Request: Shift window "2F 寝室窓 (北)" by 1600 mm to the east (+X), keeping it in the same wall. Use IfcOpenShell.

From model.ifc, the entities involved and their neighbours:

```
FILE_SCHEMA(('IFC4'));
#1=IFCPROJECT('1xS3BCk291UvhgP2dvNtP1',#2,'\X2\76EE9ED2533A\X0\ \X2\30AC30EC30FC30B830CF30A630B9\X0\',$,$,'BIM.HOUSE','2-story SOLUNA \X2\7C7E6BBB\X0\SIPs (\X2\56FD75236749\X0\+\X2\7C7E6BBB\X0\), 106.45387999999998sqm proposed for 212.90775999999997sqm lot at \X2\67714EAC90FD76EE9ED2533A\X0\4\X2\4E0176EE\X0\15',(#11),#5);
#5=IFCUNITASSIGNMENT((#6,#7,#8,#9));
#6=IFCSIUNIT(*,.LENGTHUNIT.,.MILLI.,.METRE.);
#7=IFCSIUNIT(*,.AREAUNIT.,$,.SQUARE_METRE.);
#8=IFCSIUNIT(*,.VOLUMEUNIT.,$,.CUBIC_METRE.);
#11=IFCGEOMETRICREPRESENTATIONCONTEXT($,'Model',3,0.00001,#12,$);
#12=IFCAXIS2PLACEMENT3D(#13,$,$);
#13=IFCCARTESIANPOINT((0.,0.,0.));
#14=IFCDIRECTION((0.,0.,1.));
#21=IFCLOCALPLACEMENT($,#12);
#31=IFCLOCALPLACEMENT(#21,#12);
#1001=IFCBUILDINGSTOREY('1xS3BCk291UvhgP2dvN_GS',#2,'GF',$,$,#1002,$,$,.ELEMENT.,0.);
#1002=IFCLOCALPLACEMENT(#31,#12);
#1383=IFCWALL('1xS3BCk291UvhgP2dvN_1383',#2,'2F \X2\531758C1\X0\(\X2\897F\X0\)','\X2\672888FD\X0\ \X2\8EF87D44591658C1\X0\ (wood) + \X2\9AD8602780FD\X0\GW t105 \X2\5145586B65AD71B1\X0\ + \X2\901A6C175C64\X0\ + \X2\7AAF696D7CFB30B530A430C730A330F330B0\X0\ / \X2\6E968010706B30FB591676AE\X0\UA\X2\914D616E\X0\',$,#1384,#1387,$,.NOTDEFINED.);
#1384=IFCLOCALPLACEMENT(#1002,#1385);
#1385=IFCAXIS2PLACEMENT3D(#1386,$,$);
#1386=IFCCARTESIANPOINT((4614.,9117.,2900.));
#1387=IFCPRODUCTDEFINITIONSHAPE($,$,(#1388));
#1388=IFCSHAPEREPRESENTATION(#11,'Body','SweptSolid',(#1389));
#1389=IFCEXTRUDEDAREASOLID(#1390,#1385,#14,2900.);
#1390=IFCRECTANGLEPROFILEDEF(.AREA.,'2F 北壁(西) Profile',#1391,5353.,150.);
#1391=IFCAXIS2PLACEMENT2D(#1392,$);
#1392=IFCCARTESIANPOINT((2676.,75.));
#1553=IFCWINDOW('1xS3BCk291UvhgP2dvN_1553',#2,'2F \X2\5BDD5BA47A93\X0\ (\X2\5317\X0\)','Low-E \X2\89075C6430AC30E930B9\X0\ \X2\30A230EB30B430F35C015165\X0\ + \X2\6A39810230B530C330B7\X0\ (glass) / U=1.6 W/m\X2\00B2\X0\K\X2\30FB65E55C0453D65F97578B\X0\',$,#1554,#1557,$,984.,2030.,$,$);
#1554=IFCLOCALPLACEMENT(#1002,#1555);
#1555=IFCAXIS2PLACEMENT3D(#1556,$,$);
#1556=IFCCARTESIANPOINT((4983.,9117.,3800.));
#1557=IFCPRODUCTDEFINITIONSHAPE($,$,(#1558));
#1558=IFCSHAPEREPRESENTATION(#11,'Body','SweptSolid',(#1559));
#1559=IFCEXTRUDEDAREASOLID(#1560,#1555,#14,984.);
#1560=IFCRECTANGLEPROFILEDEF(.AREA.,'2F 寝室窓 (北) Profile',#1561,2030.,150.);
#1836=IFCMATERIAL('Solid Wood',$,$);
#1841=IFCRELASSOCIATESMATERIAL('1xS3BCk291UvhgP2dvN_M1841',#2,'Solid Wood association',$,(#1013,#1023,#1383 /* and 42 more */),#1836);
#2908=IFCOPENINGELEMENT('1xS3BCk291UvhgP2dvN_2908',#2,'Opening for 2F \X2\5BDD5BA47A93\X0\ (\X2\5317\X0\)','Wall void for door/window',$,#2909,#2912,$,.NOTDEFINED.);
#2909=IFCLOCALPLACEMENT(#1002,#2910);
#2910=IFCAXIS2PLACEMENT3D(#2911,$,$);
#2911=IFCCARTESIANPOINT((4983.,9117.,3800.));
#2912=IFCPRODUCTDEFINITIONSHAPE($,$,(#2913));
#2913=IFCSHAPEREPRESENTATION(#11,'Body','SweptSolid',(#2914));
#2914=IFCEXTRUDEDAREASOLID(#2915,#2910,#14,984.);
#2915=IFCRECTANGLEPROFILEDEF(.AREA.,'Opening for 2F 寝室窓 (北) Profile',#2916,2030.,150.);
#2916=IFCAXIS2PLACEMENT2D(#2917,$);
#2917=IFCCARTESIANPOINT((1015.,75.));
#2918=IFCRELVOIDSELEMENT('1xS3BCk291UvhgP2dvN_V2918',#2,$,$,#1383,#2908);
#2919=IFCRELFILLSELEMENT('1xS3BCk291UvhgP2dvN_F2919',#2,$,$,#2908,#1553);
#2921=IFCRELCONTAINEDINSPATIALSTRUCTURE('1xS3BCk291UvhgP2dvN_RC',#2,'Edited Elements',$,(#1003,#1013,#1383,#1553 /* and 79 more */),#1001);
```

```python
import ifcopenshell
import ifcopenshell.api.geometry
import ifcopenshell.util.placement

model = ifcopenshell.open("model.ifc")

window = model.by_guid("1xS3BCk291UvhgP2dvN_1553")
opening = window.FillsVoids[0].RelatingOpeningElement
wall = opening.VoidsElements[0].RelatingBuildingElement

wall_matrix = ifcopenshell.util.placement.get_local_placement(wall.ObjectPlacement)
shift = wall_matrix[:3, 0] * 1600.0
before = ifcopenshell.util.placement.get_local_placement(window.ObjectPlacement)[:3, 3].copy()

# The window is not placed relative to its opening, so move both.
for product in (opening, window):
    matrix = ifcopenshell.util.placement.get_local_placement(product.ObjectPlacement)
    matrix[:3, 3] += shift
    ifcopenshell.api.geometry.edit_object_placement(model, product=product, matrix=matrix, is_si=False)

after = ifcopenshell.util.placement.get_local_placement(window.ObjectPlacement)[:3, 3]
print("window moved by", (after - before).round(3) + 0.0)

model.write("model-out.ifc")
```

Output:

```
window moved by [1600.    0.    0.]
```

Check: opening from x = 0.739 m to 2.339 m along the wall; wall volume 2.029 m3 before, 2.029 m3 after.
